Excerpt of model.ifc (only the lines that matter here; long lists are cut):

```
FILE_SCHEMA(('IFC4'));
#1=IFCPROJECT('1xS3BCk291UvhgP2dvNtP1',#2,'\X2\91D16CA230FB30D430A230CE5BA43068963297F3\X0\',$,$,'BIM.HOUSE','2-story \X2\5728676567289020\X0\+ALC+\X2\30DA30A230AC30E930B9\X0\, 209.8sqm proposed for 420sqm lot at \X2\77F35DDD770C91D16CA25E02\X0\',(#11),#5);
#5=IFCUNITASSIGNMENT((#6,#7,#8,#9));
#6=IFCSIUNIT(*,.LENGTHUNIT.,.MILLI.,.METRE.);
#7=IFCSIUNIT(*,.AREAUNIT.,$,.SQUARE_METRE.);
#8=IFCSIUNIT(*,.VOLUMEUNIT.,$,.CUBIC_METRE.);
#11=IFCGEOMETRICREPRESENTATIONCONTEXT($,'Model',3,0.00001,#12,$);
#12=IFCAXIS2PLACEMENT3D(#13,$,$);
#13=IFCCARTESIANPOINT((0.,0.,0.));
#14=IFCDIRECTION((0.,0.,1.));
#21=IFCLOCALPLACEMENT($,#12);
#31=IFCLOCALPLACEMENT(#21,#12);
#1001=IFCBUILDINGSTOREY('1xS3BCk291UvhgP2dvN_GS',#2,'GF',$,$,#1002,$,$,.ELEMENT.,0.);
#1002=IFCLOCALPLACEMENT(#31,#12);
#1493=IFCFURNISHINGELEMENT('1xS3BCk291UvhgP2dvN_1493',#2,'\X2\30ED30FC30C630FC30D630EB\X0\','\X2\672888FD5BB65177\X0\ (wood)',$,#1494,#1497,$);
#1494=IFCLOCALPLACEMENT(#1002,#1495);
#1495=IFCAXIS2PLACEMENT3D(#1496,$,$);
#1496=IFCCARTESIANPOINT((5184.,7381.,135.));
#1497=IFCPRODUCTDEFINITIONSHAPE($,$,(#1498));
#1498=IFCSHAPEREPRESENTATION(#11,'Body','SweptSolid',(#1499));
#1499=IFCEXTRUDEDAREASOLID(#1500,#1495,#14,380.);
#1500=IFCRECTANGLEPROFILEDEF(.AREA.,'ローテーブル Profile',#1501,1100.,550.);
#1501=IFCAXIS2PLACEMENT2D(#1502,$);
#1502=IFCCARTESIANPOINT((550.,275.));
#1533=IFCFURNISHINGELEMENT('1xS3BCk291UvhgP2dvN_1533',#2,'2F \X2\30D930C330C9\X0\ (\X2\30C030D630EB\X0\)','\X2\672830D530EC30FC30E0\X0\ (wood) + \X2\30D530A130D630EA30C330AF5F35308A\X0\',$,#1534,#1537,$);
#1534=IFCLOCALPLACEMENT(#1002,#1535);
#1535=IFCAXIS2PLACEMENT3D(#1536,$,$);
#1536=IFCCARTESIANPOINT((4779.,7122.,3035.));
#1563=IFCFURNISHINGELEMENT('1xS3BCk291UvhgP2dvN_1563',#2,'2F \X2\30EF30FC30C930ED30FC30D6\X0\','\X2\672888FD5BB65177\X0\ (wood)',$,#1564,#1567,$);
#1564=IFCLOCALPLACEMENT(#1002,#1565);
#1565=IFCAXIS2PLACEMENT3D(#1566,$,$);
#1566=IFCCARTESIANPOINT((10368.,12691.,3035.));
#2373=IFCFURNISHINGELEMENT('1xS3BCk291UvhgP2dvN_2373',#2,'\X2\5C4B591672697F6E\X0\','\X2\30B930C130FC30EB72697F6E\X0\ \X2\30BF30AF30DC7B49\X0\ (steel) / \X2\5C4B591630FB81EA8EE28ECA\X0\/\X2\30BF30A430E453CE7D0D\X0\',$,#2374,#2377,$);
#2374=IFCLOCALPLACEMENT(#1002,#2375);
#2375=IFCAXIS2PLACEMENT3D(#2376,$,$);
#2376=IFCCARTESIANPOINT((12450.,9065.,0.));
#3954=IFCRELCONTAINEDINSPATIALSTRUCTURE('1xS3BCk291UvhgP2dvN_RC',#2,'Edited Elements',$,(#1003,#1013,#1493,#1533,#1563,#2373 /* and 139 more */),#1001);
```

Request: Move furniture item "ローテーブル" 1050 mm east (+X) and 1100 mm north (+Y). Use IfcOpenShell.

```python
import ifcopenshell
import ifcopenshell.api.geometry
import ifcopenshell.util.placement
import ifcopenshell.util.unit

model = ifcopenshell.open("model.ifc")
unit_scale = ifcopenshell.util.unit.calculate_unit_scale(model)

item = model.by_guid("1xS3BCk291UvhgP2dvN_1493")
matrix = ifcopenshell.util.placement.get_local_placement(item.ObjectPlacement)
matrix[0, 3] += 1.05 / unit_scale
matrix[1, 3] += 1.1 / unit_scale
ifcopenshell.api.geometry.edit_object_placement(model, product=item, matrix=matrix, is_si=False)

print(ifcopenshell.util.placement.get_local_placement(item.ObjectPlacement).round(3) + 0.0)

model.write("model_edited.ifc")
```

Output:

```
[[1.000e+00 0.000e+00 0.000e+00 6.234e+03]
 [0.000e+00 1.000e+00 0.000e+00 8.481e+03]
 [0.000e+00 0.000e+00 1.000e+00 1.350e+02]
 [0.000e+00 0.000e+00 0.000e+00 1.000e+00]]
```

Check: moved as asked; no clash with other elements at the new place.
